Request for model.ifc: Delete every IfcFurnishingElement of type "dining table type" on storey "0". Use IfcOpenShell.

First a look at what the model holds.

```python
import ifcopenshell
import ifcopenshell.util.element

model = ifcopenshell.open("model.ifc")
print(model.schema)
storey = next(s for s in model.by_type("IfcBuildingStorey") if s.Name == "0")
furniture = [e for e in ifcopenshell.util.element.get_decomposition(storey) if e.is_a("IfcFurnishingElement")]
seen = {}
for e in furniture:
    element_type = ifcopenshell.util.element.get_type(e)
    name = element_type.Name if element_type not in (None, e) else None
    seen[name] = seen.get(name, 0) + 1
for name, count in sorted(seen.items(), key=str):
    print(count, "x", name)
```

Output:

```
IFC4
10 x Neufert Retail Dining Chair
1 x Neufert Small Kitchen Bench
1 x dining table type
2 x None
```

```python
import ifcopenshell
import ifcopenshell.api.root
import ifcopenshell.util.element

model = ifcopenshell.open("model.ifc")

storey = next(s for s in model.by_type("IfcBuildingStorey") if s.Name == "0")
furniture = [e for e in ifcopenshell.util.element.get_decomposition(storey) if e.is_a("IfcFurnishingElement")]
targets = [e for e in furniture if (t := ifcopenshell.util.element.get_type(e)) not in (None, e) and t.Name == "dining table type"]

for e in targets:
    ifcopenshell.api.root.remove_product(model, product=e)
print(len(targets), "removed")

model.write("model-out.ifc")
```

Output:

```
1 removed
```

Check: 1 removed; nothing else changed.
